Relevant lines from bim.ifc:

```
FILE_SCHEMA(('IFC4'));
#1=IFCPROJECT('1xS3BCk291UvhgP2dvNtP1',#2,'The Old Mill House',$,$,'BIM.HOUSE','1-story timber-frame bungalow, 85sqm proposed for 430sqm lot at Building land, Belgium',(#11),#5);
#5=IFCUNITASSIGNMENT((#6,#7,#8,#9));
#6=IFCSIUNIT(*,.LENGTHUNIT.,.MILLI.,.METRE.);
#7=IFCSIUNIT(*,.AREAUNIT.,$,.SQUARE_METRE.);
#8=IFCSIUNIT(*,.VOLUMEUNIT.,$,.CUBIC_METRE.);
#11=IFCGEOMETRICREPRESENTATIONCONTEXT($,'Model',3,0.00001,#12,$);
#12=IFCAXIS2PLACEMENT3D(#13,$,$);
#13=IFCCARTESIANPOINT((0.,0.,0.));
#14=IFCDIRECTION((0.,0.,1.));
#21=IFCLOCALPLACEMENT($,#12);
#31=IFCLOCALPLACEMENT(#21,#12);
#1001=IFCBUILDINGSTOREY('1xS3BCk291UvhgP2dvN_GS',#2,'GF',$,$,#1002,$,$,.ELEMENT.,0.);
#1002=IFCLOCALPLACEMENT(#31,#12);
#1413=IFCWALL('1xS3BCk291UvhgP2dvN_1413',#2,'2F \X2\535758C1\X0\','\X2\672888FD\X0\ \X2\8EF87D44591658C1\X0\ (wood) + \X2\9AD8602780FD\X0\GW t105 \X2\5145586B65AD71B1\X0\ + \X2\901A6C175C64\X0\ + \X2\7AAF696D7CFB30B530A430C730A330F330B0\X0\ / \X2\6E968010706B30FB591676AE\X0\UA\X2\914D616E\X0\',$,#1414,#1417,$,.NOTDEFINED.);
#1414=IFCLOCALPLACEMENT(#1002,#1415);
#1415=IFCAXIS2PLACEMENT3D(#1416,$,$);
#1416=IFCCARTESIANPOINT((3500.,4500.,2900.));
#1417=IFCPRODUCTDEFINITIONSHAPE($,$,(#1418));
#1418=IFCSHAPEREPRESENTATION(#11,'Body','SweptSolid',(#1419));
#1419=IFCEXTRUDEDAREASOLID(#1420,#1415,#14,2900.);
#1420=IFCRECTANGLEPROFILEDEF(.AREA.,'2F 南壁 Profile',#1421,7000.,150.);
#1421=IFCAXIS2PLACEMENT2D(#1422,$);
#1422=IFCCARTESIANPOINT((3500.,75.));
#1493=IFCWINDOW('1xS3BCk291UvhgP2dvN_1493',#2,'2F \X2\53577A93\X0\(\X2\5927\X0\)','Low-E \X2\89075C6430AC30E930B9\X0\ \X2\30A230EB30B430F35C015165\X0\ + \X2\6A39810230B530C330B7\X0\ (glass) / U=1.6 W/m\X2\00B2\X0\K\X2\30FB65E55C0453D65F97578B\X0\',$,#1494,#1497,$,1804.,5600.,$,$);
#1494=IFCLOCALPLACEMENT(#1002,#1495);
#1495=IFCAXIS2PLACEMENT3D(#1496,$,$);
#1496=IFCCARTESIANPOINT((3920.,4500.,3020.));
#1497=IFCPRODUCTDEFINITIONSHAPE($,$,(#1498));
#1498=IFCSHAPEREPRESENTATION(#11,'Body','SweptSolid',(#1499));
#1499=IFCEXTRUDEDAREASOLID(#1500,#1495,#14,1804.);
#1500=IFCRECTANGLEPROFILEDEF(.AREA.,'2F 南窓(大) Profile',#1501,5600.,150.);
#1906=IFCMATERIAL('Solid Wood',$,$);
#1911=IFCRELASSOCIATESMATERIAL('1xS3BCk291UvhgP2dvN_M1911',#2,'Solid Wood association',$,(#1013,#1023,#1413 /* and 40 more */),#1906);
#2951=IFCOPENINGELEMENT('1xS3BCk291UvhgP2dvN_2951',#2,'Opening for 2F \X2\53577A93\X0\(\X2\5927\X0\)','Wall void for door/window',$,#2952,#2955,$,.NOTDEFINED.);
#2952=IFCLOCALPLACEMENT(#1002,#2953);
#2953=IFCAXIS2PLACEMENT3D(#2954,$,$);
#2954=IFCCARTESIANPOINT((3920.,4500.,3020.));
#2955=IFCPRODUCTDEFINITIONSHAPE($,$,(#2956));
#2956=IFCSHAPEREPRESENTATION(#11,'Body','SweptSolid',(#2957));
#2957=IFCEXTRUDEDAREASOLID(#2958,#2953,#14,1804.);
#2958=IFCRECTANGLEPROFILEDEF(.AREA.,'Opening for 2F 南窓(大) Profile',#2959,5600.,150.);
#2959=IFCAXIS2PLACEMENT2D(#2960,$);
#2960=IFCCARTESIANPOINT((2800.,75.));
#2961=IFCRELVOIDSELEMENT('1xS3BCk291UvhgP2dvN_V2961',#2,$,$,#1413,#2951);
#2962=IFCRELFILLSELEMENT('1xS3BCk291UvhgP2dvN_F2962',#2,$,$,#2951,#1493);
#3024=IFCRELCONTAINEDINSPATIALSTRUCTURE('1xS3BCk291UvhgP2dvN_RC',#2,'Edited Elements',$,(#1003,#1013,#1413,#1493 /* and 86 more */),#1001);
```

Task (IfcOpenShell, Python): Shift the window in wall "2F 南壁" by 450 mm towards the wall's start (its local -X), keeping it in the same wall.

```python
import ifcopenshell
import ifcopenshell.api.geometry
import ifcopenshell.util.placement
import ifcopenshell.util.unit

model = ifcopenshell.open("bim.ifc")
unit_scale = ifcopenshell.util.unit.calculate_unit_scale(model)

window = model.by_guid("1xS3BCk291UvhgP2dvN_1493")
opening = window.FillsVoids[0].RelatingOpeningElement
wall = opening.VoidsElements[0].RelatingBuildingElement

wall_matrix = ifcopenshell.util.placement.get_local_placement(wall.ObjectPlacement)
shift = wall_matrix[:3, 0] * -0.45 / unit_scale
before = ifcopenshell.util.placement.get_local_placement(window.ObjectPlacement)[:3, 3].copy()

# The window is not placed relative to its opening, so move both.
for product in (opening, window):
    matrix = ifcopenshell.util.placement.get_local_placement(product.ObjectPlacement)
    matrix[:3, 3] += shift
    ifcopenshell.api.geometry.edit_object_placement(model, product=product, matrix=matrix, is_si=False)

after = ifcopenshell.util.placement.get_local_placement(window.ObjectPlacement)[:3, 3]
print("window moved by", (after - before).round(3) + 0.0)

model.write("bim-out.ifc")
```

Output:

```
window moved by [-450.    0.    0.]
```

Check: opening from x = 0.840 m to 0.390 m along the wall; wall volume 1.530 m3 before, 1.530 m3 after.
